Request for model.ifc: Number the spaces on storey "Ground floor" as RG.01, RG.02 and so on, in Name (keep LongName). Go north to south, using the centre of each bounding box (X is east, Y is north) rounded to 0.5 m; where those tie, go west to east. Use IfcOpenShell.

First a look at what the model holds.

```python
import ifcopenshell
import ifcopenshell.util.element
import ifcopenshell.util.placement

model = ifcopenshell.open("model.ifc")
print(model.schema)
storey = next(s for s in model.by_type("IfcBuildingStorey") if s.Name == "Ground floor")
spaces = [e for e in ifcopenshell.util.element.get_decomposition(storey) if e.is_a("IfcSpace")]
for e in sorted(spaces, key=lambda e: e.id()):
    origin = ifcopenshell.util.placement.get_local_placement(e.ObjectPlacement)[:3, 3]
    print(e.id(), e.Name, e.LongName, origin.round(2) + 0.0, sep=" | ")
```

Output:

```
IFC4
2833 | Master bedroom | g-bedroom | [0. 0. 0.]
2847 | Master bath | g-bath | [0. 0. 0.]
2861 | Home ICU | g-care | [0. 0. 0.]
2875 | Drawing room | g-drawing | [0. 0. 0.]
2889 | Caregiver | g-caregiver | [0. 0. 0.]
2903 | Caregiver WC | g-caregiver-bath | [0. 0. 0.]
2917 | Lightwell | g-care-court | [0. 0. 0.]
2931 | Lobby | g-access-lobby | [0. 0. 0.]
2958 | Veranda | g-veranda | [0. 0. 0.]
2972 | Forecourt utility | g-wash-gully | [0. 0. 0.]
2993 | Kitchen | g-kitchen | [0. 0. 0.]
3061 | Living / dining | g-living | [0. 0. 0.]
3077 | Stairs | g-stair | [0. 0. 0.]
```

```python
import ifcopenshell
import ifcopenshell.geom
import ifcopenshell.util.element
import ifcopenshell.util.shape

model = ifcopenshell.open("model.ifc")
settings = ifcopenshell.geom.settings()
settings.set("use-world-coords", True)


def centre(element):
    shape = ifcopenshell.geom.create_shape(settings, element)
    return ifcopenshell.util.shape.get_bbox_centroid(shape.geometry)


storey = next(s for s in model.by_type("IfcBuildingStorey") if s.Name == "Ground floor")
spaces = [e for e in ifcopenshell.util.element.get_decomposition(storey) if e.is_a("IfcSpace")]

# Insertion points can sit at a corner or the storey origin, so sort by the geometry (in metres).
centres = {e: centre(e) for e in spaces}
spaces.sort(key=lambda e: (-round(centres[e][1] / 0.5), centres[e][0]))

for i, e in enumerate(spaces, start=1):
    number = f"RG.{i:02d}"
    e.Name = number
    print(e.id(), number)

model.write("model-out.ifc")
```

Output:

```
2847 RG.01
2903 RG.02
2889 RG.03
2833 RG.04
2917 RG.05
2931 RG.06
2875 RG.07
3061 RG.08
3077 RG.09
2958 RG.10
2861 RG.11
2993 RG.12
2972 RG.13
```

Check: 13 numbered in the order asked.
